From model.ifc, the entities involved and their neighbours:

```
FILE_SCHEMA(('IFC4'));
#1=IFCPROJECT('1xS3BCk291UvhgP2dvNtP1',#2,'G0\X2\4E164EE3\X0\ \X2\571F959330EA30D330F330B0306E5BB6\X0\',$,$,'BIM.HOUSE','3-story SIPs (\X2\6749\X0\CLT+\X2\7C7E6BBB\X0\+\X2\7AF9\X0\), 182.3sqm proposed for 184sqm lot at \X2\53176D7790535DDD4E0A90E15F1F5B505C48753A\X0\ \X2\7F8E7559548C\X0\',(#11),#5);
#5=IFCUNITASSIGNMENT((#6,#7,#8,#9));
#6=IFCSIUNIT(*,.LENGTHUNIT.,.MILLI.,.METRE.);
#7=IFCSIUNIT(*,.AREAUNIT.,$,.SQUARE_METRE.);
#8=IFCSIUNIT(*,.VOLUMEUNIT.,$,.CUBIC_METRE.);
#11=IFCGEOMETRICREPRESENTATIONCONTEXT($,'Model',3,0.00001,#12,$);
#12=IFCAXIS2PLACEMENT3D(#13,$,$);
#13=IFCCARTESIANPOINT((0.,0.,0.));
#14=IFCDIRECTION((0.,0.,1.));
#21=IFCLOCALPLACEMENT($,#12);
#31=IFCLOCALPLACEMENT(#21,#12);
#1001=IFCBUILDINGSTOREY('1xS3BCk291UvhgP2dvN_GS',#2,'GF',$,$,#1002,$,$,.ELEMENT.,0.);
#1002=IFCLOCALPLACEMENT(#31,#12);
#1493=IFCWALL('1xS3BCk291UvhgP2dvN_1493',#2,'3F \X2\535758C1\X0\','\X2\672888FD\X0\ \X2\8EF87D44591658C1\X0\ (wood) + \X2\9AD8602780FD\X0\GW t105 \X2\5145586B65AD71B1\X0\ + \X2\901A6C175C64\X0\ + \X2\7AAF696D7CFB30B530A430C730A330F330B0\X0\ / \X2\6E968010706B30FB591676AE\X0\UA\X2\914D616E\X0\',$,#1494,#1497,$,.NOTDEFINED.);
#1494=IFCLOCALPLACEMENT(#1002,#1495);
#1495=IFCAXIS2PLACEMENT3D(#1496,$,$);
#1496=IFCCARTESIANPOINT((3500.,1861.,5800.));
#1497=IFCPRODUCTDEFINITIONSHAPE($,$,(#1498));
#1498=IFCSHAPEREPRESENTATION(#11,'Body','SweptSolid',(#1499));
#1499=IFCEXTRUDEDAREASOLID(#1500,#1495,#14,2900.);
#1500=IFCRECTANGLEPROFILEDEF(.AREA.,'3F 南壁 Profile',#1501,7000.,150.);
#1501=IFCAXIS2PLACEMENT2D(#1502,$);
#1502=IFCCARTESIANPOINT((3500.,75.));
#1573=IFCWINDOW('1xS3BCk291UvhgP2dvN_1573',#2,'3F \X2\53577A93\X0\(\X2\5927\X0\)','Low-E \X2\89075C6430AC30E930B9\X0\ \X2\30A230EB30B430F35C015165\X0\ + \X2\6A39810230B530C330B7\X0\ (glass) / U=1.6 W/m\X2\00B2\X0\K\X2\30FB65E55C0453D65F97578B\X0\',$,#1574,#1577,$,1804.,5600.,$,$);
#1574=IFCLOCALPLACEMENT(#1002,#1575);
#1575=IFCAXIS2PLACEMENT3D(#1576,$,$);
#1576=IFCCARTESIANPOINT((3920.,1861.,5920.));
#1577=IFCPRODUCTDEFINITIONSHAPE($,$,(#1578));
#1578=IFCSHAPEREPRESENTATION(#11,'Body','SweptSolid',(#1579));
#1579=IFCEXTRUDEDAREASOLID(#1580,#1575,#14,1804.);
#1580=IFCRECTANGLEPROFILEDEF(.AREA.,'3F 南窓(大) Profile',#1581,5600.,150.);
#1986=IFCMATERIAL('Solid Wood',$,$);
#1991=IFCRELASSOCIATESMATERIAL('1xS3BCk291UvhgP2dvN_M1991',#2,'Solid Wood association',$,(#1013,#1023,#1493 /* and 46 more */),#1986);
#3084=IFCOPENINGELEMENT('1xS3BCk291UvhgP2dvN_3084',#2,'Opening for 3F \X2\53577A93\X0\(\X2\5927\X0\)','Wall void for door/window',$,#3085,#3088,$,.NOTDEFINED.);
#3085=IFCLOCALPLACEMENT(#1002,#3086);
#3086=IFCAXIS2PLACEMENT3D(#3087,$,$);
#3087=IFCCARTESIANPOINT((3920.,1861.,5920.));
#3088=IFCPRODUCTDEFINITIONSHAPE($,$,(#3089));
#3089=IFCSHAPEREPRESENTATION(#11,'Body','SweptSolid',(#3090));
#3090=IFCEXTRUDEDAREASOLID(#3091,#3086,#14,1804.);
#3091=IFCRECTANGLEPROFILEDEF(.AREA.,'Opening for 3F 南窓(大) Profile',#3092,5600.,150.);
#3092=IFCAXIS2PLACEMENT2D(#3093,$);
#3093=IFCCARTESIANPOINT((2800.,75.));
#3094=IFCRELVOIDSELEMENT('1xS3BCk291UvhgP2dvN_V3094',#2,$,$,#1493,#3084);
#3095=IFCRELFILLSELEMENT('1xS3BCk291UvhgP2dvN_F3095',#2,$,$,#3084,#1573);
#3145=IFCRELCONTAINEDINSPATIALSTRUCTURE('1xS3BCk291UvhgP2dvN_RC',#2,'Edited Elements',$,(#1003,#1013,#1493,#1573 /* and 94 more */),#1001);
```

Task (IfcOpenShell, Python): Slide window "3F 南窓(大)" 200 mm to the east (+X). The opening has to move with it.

```python
import ifcopenshell
import ifcopenshell.api.geometry
import ifcopenshell.util.placement
import ifcopenshell.util.unit

model = ifcopenshell.open("model.ifc")
unit_scale = ifcopenshell.util.unit.calculate_unit_scale(model)

window = model.by_id(1573)
opening = window.FillsVoids[0].RelatingOpeningElement
wall = opening.VoidsElements[0].RelatingBuildingElement

wall_matrix = ifcopenshell.util.placement.get_local_placement(wall.ObjectPlacement)
shift = wall_matrix[:3, 0] * 0.2 / unit_scale
before = ifcopenshell.util.placement.get_local_placement(window.ObjectPlacement)[:3, 3].copy()

# The window is not placed relative to its opening, so move both.
for product in (opening, window):
    matrix = ifcopenshell.util.placement.get_local_placement(product.ObjectPlacement)
    matrix[:3, 3] += shift
    ifcopenshell.api.geometry.edit_object_placement(model, product=product, matrix=matrix, is_si=False)

after = ifcopenshell.util.placement.get_local_placement(window.ObjectPlacement)[:3, 3]
print("window moved by", (after - before).round(3) + 0.0)

model.write("model-out.ifc")
```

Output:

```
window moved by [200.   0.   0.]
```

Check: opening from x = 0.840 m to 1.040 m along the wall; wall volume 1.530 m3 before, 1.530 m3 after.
